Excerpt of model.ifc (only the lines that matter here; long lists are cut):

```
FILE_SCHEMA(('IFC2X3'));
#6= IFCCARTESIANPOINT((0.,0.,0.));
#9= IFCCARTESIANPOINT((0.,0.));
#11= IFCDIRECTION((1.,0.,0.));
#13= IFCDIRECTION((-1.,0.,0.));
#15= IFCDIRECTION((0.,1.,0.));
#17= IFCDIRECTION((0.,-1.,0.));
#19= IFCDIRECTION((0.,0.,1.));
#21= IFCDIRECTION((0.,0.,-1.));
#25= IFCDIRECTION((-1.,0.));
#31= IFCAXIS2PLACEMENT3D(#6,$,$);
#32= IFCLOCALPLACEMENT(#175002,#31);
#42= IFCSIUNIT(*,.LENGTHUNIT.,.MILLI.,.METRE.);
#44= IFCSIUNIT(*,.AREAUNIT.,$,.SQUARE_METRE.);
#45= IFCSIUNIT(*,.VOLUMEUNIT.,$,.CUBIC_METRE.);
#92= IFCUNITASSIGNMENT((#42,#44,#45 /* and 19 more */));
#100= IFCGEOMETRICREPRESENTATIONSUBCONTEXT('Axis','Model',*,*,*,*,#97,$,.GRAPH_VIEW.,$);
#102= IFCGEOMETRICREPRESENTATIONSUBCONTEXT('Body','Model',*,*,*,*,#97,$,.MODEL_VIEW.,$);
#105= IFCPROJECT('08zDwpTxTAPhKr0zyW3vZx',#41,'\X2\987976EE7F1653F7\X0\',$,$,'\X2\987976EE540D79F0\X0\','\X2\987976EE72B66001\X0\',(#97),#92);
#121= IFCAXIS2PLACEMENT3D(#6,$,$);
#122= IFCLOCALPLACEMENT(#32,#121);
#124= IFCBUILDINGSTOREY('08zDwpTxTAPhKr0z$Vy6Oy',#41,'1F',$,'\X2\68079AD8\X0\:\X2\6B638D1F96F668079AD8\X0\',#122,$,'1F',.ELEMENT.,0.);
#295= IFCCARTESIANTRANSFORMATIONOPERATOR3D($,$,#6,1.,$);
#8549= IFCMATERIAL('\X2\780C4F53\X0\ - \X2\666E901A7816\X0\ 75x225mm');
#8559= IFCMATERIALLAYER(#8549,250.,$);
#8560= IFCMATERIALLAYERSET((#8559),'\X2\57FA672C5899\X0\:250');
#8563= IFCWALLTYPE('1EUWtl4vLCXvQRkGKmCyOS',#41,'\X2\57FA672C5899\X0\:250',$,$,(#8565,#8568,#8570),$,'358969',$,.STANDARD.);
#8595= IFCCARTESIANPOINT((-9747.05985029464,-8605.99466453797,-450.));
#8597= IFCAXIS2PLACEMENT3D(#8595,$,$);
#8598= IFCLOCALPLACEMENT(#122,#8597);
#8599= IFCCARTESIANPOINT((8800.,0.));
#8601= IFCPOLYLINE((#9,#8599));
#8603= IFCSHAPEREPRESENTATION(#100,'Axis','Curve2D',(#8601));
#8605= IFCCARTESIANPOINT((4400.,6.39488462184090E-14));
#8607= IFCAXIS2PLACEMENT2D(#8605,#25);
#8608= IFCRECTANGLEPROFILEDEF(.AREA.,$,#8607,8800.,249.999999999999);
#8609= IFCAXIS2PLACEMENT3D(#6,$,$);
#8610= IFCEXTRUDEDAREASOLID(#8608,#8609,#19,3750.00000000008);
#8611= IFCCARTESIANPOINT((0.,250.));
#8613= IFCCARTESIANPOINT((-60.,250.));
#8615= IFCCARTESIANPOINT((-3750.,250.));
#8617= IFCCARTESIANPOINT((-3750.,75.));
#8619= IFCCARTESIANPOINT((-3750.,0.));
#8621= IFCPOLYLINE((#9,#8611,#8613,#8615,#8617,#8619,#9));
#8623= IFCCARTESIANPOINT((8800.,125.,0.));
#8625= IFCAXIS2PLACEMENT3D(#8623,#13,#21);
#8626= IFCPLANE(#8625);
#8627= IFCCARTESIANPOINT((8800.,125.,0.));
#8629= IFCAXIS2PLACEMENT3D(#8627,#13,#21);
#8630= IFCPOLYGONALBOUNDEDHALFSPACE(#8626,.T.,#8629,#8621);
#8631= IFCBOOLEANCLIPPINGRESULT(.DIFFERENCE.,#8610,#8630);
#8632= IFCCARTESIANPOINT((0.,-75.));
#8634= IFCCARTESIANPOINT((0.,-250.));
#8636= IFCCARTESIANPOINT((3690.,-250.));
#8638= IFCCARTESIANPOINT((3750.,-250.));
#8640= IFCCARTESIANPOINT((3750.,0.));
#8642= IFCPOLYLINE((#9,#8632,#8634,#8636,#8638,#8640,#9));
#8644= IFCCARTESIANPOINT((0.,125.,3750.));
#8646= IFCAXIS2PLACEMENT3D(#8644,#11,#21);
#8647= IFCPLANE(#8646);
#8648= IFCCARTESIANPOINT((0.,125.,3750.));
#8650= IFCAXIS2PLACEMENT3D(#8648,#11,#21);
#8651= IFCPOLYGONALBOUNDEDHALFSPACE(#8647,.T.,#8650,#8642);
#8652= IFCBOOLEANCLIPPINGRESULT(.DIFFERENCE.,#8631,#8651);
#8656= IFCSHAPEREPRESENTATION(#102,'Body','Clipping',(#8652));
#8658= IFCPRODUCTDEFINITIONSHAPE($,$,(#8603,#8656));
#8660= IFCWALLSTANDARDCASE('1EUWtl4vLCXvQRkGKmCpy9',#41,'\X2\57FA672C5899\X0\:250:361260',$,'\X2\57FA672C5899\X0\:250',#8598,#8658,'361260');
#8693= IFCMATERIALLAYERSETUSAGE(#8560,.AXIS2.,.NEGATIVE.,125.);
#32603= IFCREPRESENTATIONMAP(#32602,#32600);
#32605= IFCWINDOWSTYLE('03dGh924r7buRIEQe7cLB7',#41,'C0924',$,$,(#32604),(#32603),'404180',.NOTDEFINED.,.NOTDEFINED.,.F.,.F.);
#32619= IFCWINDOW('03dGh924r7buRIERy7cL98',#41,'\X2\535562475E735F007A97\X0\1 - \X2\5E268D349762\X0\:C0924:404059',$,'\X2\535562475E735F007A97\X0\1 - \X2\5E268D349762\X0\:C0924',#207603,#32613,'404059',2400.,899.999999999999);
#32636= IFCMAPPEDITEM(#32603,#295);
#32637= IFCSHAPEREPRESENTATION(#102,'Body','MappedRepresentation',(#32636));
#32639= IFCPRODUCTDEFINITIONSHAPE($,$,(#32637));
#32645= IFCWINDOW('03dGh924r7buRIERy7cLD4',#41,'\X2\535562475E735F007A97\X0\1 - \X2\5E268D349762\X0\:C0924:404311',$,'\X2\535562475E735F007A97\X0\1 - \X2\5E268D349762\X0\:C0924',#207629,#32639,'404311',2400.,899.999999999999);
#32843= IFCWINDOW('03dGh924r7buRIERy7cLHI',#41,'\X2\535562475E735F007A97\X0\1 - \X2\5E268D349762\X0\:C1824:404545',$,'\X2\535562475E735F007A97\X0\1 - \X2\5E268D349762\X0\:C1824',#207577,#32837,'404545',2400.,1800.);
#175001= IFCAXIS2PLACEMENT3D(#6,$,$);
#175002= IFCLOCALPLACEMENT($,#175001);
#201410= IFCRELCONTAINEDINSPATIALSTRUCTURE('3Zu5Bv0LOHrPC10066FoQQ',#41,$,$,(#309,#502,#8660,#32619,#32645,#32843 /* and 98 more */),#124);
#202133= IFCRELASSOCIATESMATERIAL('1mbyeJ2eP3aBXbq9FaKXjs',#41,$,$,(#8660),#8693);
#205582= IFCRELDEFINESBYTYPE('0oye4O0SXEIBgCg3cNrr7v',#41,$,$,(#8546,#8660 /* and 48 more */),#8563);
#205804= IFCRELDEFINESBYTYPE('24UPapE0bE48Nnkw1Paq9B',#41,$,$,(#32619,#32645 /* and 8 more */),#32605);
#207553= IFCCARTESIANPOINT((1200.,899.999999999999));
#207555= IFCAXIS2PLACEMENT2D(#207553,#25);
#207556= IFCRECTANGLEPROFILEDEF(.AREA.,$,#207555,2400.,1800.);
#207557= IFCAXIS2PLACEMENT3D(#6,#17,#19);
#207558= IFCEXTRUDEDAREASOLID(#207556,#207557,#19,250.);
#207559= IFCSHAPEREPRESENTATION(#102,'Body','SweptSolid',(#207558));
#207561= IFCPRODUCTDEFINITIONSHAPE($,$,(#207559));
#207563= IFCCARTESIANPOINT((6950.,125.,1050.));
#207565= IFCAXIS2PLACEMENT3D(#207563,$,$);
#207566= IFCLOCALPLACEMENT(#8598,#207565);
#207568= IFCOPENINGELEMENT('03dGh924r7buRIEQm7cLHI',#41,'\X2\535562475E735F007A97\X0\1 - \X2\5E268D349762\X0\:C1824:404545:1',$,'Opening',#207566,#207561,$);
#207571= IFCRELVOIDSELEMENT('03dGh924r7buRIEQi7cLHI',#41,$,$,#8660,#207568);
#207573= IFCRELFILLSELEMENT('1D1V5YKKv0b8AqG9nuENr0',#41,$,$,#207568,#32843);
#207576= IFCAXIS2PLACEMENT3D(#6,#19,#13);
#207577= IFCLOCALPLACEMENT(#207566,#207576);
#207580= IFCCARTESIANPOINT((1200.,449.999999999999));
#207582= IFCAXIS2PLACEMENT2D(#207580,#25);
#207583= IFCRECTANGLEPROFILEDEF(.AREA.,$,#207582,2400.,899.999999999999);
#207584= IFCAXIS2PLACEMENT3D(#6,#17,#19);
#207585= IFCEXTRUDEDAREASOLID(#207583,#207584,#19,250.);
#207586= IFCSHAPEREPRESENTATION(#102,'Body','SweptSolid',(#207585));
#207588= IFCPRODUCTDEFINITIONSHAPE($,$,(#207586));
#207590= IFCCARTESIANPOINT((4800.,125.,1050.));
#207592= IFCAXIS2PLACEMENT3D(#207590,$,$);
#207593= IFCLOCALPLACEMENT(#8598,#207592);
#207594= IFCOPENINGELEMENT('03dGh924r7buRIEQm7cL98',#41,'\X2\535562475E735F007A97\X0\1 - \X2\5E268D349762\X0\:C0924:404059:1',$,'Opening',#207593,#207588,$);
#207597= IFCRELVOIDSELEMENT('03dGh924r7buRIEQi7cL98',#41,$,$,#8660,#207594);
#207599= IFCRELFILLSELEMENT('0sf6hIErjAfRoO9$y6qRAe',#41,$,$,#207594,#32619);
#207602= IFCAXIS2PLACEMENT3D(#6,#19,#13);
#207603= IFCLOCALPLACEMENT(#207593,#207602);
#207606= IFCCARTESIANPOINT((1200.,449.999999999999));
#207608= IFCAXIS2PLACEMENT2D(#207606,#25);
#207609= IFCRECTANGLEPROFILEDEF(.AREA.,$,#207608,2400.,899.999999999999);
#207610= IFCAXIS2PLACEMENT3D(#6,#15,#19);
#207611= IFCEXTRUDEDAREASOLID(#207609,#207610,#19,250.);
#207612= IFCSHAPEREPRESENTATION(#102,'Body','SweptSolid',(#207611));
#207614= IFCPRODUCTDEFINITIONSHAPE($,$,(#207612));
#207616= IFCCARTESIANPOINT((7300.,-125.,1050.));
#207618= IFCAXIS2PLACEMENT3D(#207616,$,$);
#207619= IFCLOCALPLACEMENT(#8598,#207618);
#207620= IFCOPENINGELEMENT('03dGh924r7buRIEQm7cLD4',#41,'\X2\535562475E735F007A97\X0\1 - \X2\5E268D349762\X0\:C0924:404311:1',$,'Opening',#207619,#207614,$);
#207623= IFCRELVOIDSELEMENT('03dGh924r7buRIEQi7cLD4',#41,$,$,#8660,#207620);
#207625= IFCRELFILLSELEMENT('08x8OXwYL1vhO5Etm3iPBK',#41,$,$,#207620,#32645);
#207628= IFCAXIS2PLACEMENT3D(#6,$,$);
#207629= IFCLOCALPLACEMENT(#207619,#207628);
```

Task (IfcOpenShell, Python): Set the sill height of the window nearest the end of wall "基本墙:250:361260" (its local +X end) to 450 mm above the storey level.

```python
import numpy as np
import ifcopenshell
import ifcopenshell.api.geometry
import ifcopenshell.geom
import ifcopenshell.util.element
import ifcopenshell.util.placement
import ifcopenshell.util.shape
import ifcopenshell.util.unit

model = ifcopenshell.open("model.ifc")
unit_scale = ifcopenshell.util.unit.calculate_unit_scale(model)

window = model.by_guid("03dGh924r7buRIERy7cLD4")
opening = window.FillsVoids[0].RelatingOpeningElement
storey = ifcopenshell.util.element.get_container(window, ifc_class="IfcBuildingStorey")
level = ifcopenshell.util.placement.get_local_placement(storey.ObjectPlacement)[2, 3]

# The opening's origin need not be at the sill, so measure its lowest point.
shape = ifcopenshell.geom.create_shape(ifcopenshell.geom.settings(), opening)
bottom = ifcopenshell.util.shape.get_shape_bottom_elevation(shape, shape.geometry) / unit_scale
dz = level + 0.45 / unit_scale - bottom

shift = np.array([0.0, 0.0, dz])
# The window is placed relative to its opening, so it follows when the opening moves.
matrix = ifcopenshell.util.placement.get_local_placement(opening.ObjectPlacement)
matrix[:3, 3] += shift
ifcopenshell.api.geometry.edit_object_placement(
    model, product=opening, matrix=matrix, is_si=False, should_transform_children=True
)

print(f"moved by {dz * unit_scale:+.3f} m")

model.write("model_edited.ifc")
```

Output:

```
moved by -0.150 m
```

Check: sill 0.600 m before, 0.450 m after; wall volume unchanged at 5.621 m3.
